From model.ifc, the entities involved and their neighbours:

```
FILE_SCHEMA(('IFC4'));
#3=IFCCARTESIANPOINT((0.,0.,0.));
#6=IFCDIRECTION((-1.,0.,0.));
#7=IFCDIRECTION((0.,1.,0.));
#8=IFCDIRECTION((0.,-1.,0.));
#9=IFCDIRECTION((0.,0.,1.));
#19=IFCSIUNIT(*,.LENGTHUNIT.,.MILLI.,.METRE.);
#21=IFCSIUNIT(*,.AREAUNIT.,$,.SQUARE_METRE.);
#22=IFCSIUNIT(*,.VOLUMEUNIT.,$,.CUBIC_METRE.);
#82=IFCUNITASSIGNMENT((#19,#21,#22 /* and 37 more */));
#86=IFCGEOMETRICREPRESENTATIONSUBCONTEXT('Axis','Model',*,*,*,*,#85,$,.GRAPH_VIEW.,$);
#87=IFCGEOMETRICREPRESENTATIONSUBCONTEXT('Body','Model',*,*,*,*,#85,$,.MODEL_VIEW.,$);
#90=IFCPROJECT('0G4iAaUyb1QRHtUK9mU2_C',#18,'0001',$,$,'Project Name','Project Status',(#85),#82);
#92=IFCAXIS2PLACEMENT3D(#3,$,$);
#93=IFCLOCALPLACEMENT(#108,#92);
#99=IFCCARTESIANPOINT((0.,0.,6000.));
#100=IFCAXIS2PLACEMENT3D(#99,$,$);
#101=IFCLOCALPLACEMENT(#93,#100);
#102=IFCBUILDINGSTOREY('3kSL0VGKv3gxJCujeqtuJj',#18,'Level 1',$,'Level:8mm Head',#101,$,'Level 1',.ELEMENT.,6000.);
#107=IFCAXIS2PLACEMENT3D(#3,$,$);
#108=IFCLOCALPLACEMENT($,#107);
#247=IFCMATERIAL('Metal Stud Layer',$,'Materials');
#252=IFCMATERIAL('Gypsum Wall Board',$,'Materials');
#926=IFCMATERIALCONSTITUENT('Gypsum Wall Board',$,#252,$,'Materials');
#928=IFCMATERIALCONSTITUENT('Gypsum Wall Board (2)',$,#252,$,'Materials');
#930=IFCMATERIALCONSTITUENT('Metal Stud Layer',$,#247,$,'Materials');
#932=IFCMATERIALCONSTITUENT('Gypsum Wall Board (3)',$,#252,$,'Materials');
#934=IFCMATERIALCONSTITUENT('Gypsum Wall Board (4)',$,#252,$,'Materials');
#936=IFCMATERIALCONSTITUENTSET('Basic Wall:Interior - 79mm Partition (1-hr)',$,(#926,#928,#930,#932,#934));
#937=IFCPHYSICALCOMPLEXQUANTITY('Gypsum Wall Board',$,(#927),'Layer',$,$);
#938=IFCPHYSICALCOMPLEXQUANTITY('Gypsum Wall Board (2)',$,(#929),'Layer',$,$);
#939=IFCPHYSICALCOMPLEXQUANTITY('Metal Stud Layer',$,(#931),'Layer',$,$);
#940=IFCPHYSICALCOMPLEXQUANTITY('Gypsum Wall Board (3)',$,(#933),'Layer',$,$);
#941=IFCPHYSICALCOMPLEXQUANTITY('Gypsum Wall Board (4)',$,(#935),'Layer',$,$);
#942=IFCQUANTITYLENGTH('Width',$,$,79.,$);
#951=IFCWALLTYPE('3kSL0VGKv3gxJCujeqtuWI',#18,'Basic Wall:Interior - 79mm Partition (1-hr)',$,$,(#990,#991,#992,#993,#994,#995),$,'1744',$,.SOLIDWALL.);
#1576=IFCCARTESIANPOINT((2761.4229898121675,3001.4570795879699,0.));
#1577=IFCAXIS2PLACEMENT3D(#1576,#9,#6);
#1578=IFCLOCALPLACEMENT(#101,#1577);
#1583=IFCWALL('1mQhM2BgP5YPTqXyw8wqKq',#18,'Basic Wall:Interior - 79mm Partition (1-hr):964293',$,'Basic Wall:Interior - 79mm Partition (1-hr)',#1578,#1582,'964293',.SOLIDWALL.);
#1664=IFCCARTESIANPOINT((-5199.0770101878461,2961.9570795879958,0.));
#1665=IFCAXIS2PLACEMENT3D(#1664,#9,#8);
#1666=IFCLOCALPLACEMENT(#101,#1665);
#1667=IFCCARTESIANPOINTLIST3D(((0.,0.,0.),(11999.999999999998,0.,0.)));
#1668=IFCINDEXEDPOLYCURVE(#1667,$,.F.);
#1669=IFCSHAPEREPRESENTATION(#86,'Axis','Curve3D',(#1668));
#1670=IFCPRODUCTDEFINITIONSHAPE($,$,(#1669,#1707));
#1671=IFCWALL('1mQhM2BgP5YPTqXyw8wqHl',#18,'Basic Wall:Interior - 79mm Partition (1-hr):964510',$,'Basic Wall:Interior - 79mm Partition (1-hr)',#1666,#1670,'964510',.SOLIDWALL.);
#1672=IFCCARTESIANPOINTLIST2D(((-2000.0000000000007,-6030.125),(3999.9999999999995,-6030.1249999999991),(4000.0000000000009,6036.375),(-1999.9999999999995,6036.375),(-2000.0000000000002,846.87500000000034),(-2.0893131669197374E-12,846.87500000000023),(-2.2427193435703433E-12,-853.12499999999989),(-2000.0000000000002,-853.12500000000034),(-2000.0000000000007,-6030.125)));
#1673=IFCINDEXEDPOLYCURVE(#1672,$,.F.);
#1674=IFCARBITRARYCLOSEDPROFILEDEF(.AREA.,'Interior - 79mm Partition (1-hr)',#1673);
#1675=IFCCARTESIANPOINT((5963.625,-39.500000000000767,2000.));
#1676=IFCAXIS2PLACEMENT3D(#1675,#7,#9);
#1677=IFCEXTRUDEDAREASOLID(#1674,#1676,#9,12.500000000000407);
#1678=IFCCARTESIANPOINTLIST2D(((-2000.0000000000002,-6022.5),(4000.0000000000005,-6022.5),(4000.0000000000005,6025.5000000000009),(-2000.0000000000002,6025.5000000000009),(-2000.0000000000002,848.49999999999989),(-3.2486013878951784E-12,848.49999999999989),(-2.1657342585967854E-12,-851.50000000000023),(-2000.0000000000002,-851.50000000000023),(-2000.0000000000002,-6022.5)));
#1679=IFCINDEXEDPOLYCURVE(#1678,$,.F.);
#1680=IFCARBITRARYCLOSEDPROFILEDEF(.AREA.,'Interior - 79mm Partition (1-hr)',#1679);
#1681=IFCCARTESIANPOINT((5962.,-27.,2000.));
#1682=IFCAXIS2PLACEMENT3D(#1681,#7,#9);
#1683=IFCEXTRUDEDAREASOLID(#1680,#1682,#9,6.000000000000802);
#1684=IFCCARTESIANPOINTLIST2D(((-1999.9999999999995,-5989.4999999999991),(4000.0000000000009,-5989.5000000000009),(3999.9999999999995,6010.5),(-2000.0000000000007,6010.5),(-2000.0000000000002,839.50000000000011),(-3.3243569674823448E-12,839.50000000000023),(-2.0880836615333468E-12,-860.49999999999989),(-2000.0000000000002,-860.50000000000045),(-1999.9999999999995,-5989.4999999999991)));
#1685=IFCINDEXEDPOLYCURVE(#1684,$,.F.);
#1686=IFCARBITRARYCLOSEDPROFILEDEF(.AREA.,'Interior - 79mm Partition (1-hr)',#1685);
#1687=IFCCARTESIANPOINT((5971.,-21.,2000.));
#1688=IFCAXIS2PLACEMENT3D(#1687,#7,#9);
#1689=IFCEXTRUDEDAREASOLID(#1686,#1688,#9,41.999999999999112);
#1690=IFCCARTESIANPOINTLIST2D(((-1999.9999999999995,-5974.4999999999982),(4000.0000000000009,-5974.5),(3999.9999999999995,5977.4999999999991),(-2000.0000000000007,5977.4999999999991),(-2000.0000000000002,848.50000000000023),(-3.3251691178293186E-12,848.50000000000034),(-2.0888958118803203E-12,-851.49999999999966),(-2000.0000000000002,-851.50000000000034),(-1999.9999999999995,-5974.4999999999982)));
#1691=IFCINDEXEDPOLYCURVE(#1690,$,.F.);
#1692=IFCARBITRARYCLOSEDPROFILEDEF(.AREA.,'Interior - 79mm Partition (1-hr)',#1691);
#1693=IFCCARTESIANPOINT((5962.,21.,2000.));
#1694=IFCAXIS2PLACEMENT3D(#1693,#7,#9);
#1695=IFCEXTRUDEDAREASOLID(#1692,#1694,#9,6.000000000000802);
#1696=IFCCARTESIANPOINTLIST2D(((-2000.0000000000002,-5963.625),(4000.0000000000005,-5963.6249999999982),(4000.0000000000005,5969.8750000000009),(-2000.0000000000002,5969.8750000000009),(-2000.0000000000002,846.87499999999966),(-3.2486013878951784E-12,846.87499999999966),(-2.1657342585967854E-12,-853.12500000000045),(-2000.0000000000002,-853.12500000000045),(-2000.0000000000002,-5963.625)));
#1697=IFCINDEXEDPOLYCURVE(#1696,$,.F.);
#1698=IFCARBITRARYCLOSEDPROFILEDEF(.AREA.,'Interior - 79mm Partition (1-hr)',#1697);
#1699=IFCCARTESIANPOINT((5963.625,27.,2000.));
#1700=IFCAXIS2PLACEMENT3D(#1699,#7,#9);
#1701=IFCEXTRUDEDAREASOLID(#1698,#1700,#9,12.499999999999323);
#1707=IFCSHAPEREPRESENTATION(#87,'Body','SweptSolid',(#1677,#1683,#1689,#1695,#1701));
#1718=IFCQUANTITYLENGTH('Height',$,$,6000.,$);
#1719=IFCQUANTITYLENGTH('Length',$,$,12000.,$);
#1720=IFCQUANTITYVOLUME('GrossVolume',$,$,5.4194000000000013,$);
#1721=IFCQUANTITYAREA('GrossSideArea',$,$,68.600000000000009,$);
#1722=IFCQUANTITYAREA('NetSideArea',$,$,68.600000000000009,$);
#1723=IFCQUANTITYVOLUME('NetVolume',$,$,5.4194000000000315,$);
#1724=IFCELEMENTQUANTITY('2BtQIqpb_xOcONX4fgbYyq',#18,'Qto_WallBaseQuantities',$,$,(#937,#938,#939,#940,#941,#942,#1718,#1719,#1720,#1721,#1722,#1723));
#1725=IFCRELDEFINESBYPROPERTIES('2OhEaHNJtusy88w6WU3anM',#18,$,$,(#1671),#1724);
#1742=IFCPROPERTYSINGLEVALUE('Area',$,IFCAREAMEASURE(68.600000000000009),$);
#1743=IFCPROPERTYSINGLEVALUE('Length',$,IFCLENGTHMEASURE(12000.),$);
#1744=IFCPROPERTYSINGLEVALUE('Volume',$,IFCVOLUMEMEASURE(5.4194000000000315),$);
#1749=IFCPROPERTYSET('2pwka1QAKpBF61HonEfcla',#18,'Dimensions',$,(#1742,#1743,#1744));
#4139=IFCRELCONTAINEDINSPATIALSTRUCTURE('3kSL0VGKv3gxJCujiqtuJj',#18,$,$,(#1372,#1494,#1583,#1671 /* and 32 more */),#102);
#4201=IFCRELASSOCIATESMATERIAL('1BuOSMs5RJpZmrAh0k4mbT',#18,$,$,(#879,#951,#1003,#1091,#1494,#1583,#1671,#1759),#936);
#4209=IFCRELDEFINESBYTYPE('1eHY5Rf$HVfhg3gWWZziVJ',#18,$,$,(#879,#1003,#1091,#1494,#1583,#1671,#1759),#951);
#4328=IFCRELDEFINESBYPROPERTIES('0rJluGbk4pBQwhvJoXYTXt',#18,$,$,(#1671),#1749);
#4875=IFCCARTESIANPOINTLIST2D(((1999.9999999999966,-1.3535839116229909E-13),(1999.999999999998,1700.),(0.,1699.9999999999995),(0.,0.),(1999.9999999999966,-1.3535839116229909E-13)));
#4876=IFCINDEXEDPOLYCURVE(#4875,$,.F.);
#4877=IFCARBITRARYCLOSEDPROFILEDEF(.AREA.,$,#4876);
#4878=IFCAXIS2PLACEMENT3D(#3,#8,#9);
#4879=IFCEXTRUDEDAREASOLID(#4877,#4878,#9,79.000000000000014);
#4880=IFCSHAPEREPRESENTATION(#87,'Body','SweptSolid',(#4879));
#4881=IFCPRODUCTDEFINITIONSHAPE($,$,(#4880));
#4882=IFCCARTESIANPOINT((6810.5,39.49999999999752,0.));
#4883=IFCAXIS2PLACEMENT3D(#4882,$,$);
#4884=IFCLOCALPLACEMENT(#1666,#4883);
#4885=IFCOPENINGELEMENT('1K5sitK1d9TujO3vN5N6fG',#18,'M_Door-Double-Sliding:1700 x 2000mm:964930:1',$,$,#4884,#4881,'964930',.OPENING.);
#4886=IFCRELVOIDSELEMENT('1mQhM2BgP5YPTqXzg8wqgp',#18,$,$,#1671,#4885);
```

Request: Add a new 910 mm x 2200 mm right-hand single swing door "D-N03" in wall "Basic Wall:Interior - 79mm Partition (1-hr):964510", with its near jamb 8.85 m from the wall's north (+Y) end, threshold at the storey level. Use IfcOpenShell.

```python
import numpy as np
import ifcopenshell
import ifcopenshell.api.feature
import ifcopenshell.api.geometry
import ifcopenshell.api.pset
import ifcopenshell.api.root
import ifcopenshell.api.spatial
import ifcopenshell.geom
import ifcopenshell.util.element
import ifcopenshell.util.placement
import ifcopenshell.util.representation
import ifcopenshell.util.shape
import ifcopenshell.util.unit

model = ifcopenshell.open("model.ifc")
unit_scale = ifcopenshell.util.unit.calculate_unit_scale(model)
area_scale = ifcopenshell.util.unit.calculate_unit_scale(model, "AREAUNIT")
volume_scale = ifcopenshell.util.unit.calculate_unit_scale(model, "VOLUMEUNIT")
settings = ifcopenshell.geom.settings()


def volume(element):
    """Net volume in cubic metres, openings subtracted."""
    shape = ifcopenshell.geom.create_shape(settings, element)
    return ifcopenshell.util.shape.get_volume(shape.geometry)


wall = model.by_guid("1mQhM2BgP5YPTqXyw8wqHl")
storey = ifcopenshell.util.element.get_container(wall, ifc_class="IfcBuildingStorey")
context = ifcopenshell.util.representation.get_context(model, "Model", "Body", "MODEL_VIEW")
before = volume(wall)

width, height, from_end, sill = 0.91, 2.2, 8.85, 0.0  # metres

# The wall runs along its own X axis, and the end named is its -X end.
wall_shape = ifcopenshell.geom.create_shape(settings, wall)
x, y, z = ifcopenshell.util.shape.get_vertices(wall_shape.geometry).T
start = x.min() + from_end
face, thickness = float(y.min()), float(y.max() - y.min())
wall_matrix = ifcopenshell.util.placement.get_local_placement(wall.ObjectPlacement)
level = ifcopenshell.util.placement.get_local_placement(storey.ObjectPlacement)[2, 3]


def in_wall(x, y):
    """Placement at x, y metres in the wall's axes, at sill height."""
    matrix = wall_matrix.copy()
    matrix[:, 3] = wall_matrix @ np.array([x / unit_scale, y / unit_scale, 0.0, 1.0])
    matrix[2, 3] = level + sill / unit_scale
    return matrix


# Opening: a box that overshoots both wall faces by 50 mm.
opening = ifcopenshell.api.root.create_entity(model, ifc_class="IfcOpeningElement", predefined_type="OPENING")
box = ifcopenshell.api.geometry.add_wall_representation(
    model, context=context, length=width, height=height, thickness=thickness + 0.1
)
ifcopenshell.api.geometry.assign_representation(model, product=opening, representation=box)
ifcopenshell.api.geometry.edit_object_placement(model, product=opening, matrix=in_wall(start, face - 0.05), is_si=False)
ifcopenshell.api.feature.add_feature(model, feature=opening, element=wall)

door = ifcopenshell.api.root.create_entity(model, ifc_class="IfcDoor", name="D-N03", predefined_type="DOOR")
door.OverallWidth, door.OverallHeight = width / unit_scale, height / unit_scale
door.OperationType = "SINGLE_SWING_RIGHT"
body = ifcopenshell.api.geometry.add_door_representation(
    model,
    context=context,
    overall_width=door.OverallWidth,
    overall_height=door.OverallHeight,
    operation_type="SINGLE_SWING_RIGHT",
    lining_properties={"LiningDepth": thickness / unit_scale, "ThresholdDepth": thickness / unit_scale},
)
ifcopenshell.api.geometry.assign_representation(model, product=door, representation=body)
ifcopenshell.api.spatial.assign_container(model, products=[door], relating_structure=storey)
ifcopenshell.api.feature.add_filling(model, opening=opening, element=door)

# The lining spans the wall, so the door starts at the wall face.
ifcopenshell.api.geometry.edit_object_placement(model, product=door, matrix=in_wall(start, face), is_si=False)

after = volume(wall)

# Update the wall's stored quantities.
qto = model.by_id(ifcopenshell.util.element.get_pset(wall, "Qto_WallBaseQuantities", should_inherit=False)["id"])
ifcopenshell.api.pset.edit_qto(model, qto=qto, properties={
    "NetSideArea": after / thickness / area_scale,
    "NetVolume": after / volume_scale,
})
pset = model.by_id(ifcopenshell.util.element.get_pset(wall, "Dimensions", should_inherit=False)["id"])
ifcopenshell.api.pset.edit_pset(model, pset=pset, properties={
    "Area": model.create_entity("IfcAreaMeasure", after / thickness / area_scale),
    "Volume": model.create_entity("IfcVolumeMeasure", after / volume_scale),
})

print(f"wall volume {before:.3f} -> {after:.3f} m3")

model.write("model_edited.ifc")
```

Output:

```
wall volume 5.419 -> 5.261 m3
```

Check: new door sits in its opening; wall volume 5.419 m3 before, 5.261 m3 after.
